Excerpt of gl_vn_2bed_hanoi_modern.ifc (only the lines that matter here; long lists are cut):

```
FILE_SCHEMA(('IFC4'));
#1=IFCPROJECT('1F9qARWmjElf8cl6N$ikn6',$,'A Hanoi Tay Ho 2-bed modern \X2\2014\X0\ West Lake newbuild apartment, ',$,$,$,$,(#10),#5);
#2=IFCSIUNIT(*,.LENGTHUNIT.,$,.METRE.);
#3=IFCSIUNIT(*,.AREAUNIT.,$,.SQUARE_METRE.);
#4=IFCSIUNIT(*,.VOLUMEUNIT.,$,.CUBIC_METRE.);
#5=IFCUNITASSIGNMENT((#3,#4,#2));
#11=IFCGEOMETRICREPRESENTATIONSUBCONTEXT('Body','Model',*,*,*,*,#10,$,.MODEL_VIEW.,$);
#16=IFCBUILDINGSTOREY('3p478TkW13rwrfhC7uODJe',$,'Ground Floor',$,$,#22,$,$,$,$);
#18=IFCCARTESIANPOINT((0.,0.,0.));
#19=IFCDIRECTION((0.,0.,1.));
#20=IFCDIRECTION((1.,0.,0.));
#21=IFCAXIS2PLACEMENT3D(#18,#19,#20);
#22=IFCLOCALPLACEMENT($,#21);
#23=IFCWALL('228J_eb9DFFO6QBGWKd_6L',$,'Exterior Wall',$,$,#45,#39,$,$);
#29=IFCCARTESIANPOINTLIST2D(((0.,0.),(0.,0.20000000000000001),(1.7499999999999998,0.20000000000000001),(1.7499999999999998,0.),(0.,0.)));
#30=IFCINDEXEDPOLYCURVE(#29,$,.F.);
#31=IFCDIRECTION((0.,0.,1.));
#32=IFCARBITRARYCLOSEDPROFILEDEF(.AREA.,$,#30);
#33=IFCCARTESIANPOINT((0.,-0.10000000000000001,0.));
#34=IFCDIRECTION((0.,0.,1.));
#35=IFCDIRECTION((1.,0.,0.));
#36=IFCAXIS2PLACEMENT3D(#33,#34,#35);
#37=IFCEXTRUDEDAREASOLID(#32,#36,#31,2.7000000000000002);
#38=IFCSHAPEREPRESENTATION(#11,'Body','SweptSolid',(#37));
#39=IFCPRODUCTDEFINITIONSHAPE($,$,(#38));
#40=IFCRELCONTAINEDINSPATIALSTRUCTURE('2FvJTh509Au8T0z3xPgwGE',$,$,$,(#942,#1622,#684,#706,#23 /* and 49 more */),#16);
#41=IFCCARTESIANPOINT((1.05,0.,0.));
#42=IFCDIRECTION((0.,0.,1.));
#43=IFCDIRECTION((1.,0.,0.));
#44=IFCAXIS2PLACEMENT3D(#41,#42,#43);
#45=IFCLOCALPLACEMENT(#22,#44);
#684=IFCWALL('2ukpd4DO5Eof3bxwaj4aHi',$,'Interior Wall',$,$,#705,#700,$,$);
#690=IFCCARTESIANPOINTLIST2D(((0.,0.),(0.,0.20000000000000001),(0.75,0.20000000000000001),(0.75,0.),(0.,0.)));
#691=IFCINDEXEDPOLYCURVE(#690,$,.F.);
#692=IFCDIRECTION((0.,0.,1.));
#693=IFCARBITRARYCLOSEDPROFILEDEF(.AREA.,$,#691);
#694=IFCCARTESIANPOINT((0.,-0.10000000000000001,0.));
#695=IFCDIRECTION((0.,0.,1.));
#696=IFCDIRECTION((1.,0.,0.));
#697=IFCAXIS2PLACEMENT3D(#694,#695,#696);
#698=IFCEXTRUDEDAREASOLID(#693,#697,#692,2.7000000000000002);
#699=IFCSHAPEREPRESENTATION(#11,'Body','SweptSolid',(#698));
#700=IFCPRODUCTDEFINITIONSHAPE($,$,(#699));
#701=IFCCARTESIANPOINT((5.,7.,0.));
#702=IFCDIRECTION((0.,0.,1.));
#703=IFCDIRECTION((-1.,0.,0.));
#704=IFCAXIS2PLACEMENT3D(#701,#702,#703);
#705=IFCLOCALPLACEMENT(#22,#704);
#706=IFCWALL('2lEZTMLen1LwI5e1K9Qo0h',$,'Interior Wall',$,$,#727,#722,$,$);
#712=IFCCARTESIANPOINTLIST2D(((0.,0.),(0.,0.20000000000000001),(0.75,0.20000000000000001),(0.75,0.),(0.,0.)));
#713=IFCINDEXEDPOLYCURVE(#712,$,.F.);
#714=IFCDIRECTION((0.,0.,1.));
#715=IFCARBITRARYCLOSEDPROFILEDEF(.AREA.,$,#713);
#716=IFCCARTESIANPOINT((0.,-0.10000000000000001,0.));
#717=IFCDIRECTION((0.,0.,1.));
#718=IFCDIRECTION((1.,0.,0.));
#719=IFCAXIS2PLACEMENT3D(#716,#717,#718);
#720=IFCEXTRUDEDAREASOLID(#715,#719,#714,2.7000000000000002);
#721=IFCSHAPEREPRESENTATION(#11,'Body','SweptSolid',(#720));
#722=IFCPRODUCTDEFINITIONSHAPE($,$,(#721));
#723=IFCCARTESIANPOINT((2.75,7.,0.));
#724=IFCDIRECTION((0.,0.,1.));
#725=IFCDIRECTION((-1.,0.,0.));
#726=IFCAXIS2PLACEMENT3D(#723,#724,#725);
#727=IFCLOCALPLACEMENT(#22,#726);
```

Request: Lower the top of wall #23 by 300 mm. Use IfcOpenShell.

```python
import ifcopenshell
import ifcopenshell.geom
import ifcopenshell.util.representation
import ifcopenshell.util.shape
import ifcopenshell.util.unit

model = ifcopenshell.open("gl_vn_2bed_hanoi_modern.ifc")
unit_scale = ifcopenshell.util.unit.calculate_unit_scale(model)
settings = ifcopenshell.geom.settings()


def volume(element):
    """Net volume in cubic metres, openings subtracted."""
    shape = ifcopenshell.geom.create_shape(settings, element)
    return ifcopenshell.util.shape.get_volume(shape.geometry)


wall = model.by_guid("228J_eb9DFFO6QBGWKd_6L")
before = volume(wall)

body = ifcopenshell.util.representation.get_representation(wall, "Model", "Body")
solid = body.Items[0]
old_height = solid.Depth
solid.Depth -= 0.3 / unit_scale
after = volume(wall)

print(f"height {old_height:g} -> {solid.Depth:g}, volume {before:.3f} -> {after:.3f} m3")

model.write("gl_vn_2bed_hanoi_modern_rev.ifc")
```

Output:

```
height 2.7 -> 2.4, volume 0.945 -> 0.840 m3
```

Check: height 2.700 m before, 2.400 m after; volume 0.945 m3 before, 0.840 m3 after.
